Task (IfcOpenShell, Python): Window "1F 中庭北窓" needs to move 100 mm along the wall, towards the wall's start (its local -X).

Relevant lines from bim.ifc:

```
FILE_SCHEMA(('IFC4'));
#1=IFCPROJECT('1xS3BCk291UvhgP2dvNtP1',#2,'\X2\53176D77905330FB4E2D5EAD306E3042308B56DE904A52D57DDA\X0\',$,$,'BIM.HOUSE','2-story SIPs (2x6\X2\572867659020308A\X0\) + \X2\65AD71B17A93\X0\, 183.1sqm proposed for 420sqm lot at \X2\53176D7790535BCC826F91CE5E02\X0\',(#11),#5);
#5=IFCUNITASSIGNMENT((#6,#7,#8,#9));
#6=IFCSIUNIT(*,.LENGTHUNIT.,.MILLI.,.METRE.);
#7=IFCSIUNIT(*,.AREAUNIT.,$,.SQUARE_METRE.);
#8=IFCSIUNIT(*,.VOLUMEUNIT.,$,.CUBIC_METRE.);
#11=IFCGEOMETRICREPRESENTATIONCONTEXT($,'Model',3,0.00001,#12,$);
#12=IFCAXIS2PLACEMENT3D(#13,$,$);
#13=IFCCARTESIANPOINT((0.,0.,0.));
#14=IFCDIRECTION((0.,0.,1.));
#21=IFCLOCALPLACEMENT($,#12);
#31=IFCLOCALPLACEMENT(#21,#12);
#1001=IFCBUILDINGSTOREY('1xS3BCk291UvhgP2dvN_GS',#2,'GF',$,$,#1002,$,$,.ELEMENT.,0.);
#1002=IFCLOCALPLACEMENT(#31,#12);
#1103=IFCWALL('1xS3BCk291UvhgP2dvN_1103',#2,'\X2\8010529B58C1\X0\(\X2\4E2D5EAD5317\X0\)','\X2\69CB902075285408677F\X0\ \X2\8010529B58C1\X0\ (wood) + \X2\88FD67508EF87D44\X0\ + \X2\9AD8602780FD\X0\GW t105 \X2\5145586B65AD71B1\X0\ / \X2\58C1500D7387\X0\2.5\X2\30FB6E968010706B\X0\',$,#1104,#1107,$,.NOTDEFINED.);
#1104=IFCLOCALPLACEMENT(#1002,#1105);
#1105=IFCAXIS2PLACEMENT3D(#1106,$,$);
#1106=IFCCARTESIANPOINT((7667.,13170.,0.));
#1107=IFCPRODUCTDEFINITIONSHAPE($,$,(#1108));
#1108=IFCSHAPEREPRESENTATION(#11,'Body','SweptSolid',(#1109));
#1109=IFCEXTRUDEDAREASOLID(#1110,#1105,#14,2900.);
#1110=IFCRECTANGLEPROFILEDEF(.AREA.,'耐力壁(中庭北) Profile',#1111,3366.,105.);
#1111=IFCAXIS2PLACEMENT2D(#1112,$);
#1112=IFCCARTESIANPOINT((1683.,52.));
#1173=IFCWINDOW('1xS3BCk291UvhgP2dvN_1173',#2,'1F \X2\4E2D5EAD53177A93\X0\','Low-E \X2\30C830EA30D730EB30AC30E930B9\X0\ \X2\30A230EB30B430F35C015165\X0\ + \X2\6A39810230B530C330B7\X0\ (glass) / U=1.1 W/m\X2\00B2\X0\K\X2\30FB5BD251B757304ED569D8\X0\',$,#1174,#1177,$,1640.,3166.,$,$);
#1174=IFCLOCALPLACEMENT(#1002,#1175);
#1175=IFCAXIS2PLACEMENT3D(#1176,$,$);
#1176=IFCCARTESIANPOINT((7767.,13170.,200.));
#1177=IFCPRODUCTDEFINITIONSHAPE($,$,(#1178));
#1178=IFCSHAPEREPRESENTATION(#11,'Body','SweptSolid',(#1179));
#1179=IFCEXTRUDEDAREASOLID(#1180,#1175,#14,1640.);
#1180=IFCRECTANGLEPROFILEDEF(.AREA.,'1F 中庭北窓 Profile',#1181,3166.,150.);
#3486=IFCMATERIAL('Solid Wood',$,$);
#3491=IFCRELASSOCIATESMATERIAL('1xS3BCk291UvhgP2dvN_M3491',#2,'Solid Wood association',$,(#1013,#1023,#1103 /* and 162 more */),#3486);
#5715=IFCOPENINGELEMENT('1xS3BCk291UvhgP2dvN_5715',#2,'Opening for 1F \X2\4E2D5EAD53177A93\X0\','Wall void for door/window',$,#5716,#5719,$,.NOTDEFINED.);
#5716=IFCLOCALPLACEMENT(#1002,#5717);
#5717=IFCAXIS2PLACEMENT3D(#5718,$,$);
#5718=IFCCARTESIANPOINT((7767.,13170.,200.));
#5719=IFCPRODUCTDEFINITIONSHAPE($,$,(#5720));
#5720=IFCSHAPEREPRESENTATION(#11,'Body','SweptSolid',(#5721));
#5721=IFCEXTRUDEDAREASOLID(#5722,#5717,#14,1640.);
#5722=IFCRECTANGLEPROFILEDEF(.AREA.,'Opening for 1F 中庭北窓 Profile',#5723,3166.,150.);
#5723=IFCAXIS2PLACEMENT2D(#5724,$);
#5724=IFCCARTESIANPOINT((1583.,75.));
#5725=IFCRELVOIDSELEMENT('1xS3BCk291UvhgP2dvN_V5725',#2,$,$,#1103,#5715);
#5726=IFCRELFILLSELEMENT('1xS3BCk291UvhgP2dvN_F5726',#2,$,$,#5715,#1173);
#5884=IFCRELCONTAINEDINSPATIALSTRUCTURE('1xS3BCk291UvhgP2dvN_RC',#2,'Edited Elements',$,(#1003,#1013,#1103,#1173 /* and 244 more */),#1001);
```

```python
import ifcopenshell
import ifcopenshell.api.geometry
import ifcopenshell.util.placement

model = ifcopenshell.open("bim.ifc")

window = model.by_guid("1xS3BCk291UvhgP2dvN_1173")
opening = window.FillsVoids[0].RelatingOpeningElement
wall = opening.VoidsElements[0].RelatingBuildingElement

wall_matrix = ifcopenshell.util.placement.get_local_placement(wall.ObjectPlacement)
shift = wall_matrix[:3, 0] * -100.0
before = ifcopenshell.util.placement.get_local_placement(window.ObjectPlacement)[:3, 3].copy()

# The window is not placed relative to its opening, so move both.
for product in (opening, window):
    matrix = ifcopenshell.util.placement.get_local_placement(product.ObjectPlacement)
    matrix[:3, 3] += shift
    ifcopenshell.api.geometry.edit_object_placement(model, product=product, matrix=matrix, is_si=False)

after = ifcopenshell.util.placement.get_local_placement(window.ObjectPlacement)[:3, 3]
print("window moved by", (after - before).round(3) + 0.0)

model.write("bim_updated.ifc")
```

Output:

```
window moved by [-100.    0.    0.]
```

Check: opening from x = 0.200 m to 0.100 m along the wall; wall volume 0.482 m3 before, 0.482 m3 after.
